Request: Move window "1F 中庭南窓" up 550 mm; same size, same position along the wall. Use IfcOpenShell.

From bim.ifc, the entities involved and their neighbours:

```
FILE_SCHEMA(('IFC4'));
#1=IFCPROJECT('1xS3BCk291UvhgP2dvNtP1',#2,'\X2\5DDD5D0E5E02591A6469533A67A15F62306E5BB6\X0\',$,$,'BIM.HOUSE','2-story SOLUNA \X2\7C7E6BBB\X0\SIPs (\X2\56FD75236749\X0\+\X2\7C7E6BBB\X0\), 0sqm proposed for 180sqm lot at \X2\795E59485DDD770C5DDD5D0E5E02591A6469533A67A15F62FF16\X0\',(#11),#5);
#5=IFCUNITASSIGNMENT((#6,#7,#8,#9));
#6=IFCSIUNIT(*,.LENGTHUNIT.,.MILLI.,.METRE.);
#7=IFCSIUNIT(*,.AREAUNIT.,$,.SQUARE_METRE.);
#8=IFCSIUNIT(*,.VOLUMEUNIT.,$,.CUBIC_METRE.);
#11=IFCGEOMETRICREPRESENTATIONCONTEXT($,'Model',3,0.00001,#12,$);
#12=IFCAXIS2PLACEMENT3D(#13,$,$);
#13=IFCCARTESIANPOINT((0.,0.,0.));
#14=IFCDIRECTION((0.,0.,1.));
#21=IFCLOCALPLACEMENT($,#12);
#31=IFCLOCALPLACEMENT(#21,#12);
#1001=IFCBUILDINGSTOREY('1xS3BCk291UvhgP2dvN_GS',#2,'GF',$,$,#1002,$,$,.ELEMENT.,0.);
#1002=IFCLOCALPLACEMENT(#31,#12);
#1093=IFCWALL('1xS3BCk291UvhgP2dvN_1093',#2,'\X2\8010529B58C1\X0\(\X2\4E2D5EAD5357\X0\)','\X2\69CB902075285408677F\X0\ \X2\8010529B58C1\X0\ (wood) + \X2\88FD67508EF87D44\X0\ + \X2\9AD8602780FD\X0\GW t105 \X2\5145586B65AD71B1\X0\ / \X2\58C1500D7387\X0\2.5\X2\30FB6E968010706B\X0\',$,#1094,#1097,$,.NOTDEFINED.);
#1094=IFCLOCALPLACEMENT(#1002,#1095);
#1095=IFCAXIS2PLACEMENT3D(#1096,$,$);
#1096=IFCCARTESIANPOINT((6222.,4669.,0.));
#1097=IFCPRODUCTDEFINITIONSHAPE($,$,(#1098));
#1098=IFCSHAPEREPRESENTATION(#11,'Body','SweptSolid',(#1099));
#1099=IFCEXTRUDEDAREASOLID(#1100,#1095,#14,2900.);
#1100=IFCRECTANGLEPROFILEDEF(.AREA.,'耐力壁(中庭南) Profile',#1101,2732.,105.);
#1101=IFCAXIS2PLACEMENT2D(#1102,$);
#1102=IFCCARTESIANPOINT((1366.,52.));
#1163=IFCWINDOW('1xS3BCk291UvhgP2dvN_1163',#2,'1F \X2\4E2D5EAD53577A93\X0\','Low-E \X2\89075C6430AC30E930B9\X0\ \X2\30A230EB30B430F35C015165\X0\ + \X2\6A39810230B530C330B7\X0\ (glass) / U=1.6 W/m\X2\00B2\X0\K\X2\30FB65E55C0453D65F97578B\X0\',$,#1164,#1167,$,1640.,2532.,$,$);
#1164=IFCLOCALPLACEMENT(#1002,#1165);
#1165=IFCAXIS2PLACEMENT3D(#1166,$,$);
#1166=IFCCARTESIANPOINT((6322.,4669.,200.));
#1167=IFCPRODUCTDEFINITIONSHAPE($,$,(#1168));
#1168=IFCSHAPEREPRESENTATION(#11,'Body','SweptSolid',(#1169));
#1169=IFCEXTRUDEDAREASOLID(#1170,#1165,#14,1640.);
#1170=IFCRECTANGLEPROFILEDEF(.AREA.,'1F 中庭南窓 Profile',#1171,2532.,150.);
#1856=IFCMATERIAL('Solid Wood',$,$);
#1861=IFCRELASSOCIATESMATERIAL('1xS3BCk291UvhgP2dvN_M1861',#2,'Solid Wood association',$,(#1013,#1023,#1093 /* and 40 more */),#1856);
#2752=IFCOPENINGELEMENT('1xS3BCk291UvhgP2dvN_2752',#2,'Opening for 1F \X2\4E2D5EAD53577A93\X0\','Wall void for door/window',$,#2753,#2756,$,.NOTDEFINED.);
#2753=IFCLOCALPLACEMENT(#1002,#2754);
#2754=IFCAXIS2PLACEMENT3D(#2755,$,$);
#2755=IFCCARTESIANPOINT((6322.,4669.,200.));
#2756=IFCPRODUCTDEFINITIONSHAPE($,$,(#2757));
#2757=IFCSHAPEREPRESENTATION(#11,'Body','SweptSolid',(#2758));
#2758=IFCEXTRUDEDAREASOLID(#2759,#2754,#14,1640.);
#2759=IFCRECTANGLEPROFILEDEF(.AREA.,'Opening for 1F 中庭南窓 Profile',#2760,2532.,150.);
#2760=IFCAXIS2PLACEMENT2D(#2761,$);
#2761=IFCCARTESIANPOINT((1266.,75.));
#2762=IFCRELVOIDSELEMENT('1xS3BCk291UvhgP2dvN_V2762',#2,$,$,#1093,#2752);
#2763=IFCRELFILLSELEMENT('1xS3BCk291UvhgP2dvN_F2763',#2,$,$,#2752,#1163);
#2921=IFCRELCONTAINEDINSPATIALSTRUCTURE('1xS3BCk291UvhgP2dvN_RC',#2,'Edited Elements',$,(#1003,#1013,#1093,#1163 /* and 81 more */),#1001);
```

```python
import numpy as np
import ifcopenshell
import ifcopenshell.api.geometry
import ifcopenshell.util.placement
import ifcopenshell.util.unit

model = ifcopenshell.open("bim.ifc")
unit_scale = ifcopenshell.util.unit.calculate_unit_scale(model)

window = model.by_id(1163)
opening = window.FillsVoids[0].RelatingOpeningElement
dz = 550.0

shift = np.array([0.0, 0.0, dz])
# The window is not placed relative to its opening, so move both.
for product in (opening, window):
    matrix = ifcopenshell.util.placement.get_local_placement(product.ObjectPlacement)
    matrix[:3, 3] += shift
    ifcopenshell.api.geometry.edit_object_placement(model, product=product, matrix=matrix, is_si=False)

print(f"moved by {dz * unit_scale:+.3f} m")

model.write("bim_v2.ifc")
```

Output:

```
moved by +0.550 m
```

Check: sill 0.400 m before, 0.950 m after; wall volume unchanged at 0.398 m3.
